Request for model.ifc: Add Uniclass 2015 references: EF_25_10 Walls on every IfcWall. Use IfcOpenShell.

First a look at what the model holds.

```python
import ifcopenshell

model = ifcopenshell.open("model.ifc")
print(model.schema)
print("classifications:", [c.Name for c in model.by_type("IfcClassification")])
for ifc_class in ("IfcDoor", "IfcRoof", "IfcStair", "IfcWall", "IfcWindow"):
    print(ifc_class, len(model.by_type(ifc_class)))
```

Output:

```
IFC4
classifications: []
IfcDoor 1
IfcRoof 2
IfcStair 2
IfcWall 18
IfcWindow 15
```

```python
import ifcopenshell
import ifcopenshell.api.classification

model = ifcopenshell.open("model.ifc")

system = ifcopenshell.api.classification.add_classification(model, classification="Uniclass 2015")

codes = {
    "IfcWall": ("EF_25_10", "Walls"),
}
for ifc_class, (code, name) in codes.items():
    products = model.by_type(ifc_class)
    ifcopenshell.api.classification.add_reference(
        model, products=products, classification=system, identification=code, name=name
    )
    print(code, len(products))

model.write("model_rev.ifc")
```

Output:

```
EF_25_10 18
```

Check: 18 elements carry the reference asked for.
